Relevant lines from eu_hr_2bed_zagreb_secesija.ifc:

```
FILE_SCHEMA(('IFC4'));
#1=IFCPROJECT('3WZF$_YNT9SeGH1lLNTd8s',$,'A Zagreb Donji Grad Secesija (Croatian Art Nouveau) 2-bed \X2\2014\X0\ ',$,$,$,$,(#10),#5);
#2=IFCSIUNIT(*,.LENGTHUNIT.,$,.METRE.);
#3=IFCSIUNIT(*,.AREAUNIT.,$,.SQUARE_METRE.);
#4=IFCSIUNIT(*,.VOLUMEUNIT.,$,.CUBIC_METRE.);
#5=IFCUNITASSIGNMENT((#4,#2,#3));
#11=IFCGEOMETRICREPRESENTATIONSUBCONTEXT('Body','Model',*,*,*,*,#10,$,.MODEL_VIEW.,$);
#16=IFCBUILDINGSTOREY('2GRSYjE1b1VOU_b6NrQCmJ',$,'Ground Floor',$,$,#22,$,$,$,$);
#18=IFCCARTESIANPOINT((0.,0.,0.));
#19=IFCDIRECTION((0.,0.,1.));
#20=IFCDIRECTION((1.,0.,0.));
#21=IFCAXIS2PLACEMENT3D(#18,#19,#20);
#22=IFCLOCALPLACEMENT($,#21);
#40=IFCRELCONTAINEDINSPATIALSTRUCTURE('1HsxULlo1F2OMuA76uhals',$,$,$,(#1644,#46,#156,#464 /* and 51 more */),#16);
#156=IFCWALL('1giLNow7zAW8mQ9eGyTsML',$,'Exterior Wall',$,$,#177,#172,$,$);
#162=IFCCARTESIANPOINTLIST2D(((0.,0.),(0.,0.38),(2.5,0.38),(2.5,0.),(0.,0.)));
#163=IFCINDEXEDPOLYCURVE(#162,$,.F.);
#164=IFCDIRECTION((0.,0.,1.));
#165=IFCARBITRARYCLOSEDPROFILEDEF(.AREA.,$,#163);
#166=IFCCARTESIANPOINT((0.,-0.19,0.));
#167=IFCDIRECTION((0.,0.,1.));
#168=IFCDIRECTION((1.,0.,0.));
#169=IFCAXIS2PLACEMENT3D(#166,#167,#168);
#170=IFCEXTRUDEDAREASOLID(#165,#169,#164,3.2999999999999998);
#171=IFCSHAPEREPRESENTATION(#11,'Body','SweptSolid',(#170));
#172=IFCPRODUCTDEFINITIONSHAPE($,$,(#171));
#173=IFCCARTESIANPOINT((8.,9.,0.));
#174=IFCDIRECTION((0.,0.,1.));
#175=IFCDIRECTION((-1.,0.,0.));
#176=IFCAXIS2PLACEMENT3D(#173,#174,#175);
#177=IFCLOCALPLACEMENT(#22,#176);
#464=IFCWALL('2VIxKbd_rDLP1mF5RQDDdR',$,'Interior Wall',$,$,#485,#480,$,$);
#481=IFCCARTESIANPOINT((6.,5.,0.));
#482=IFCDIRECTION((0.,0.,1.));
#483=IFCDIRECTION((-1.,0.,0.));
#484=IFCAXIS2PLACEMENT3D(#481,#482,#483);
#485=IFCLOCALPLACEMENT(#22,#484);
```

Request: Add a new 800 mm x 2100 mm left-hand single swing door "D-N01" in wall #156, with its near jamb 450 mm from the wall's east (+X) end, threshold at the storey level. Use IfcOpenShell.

```python
import numpy as np
import ifcopenshell
import ifcopenshell.api.feature
import ifcopenshell.api.geometry
import ifcopenshell.api.root
import ifcopenshell.api.spatial
import ifcopenshell.geom
import ifcopenshell.util.element
import ifcopenshell.util.placement
import ifcopenshell.util.representation
import ifcopenshell.util.shape
import ifcopenshell.util.unit

model = ifcopenshell.open("eu_hr_2bed_zagreb_secesija.ifc")
unit_scale = ifcopenshell.util.unit.calculate_unit_scale(model)
settings = ifcopenshell.geom.settings()


def volume(element):
    """Net volume in cubic metres, openings subtracted."""
    shape = ifcopenshell.geom.create_shape(settings, element)
    return ifcopenshell.util.shape.get_volume(shape.geometry)


wall = model.by_guid("1giLNow7zAW8mQ9eGyTsML")
storey = ifcopenshell.util.element.get_container(wall, ifc_class="IfcBuildingStorey")
context = ifcopenshell.util.representation.get_context(model, "Model", "Body", "MODEL_VIEW")
before = volume(wall)

width, height, from_end, sill = 0.8, 2.1, 0.45, 0.0  # metres

# The wall runs along its own X axis, and the end named is its -X end.
wall_shape = ifcopenshell.geom.create_shape(settings, wall)
x, y, z = ifcopenshell.util.shape.get_vertices(wall_shape.geometry).T
start = x.min() + from_end
face, thickness = float(y.min()), float(y.max() - y.min())
wall_matrix = ifcopenshell.util.placement.get_local_placement(wall.ObjectPlacement)
level = ifcopenshell.util.placement.get_local_placement(storey.ObjectPlacement)[2, 3]


def in_wall(x, y):
    """Placement at x, y metres in the wall's axes, at sill height."""
    matrix = wall_matrix.copy()
    matrix[:, 3] = wall_matrix @ np.array([x / unit_scale, y / unit_scale, 0.0, 1.0])
    matrix[2, 3] = level + sill / unit_scale
    return matrix


# Opening: a box that overshoots both wall faces by 50 mm.
opening = ifcopenshell.api.root.create_entity(model, ifc_class="IfcOpeningElement", predefined_type="OPENING")
box = ifcopenshell.api.geometry.add_wall_representation(
    model, context=context, length=width, height=height, thickness=thickness + 0.1
)
ifcopenshell.api.geometry.assign_representation(model, product=opening, representation=box)
ifcopenshell.api.geometry.edit_object_placement(model, product=opening, matrix=in_wall(start, face - 0.05), is_si=False)
ifcopenshell.api.feature.add_feature(model, feature=opening, element=wall)

door = ifcopenshell.api.root.create_entity(model, ifc_class="IfcDoor", name="D-N01", predefined_type="DOOR")
door.OverallWidth, door.OverallHeight = width / unit_scale, height / unit_scale
door.OperationType = "SINGLE_SWING_LEFT"
body = ifcopenshell.api.geometry.add_door_representation(
    model,
    context=context,
    overall_width=door.OverallWidth,
    overall_height=door.OverallHeight,
    operation_type="SINGLE_SWING_LEFT",
    lining_properties={"LiningDepth": thickness / unit_scale, "ThresholdDepth": thickness / unit_scale},
)
ifcopenshell.api.geometry.assign_representation(model, product=door, representation=body)
ifcopenshell.api.spatial.assign_container(model, products=[door], relating_structure=storey)
ifcopenshell.api.feature.add_filling(model, opening=opening, element=door)

# The lining spans the wall, so the door starts at the wall face.
ifcopenshell.api.geometry.edit_object_placement(model, product=door, matrix=in_wall(start, face), is_si=False)

after = volume(wall)

print(f"wall volume {before:.3f} -> {after:.3f} m3")

model.write("eu_hr_2bed_zagreb_secesija-out.ifc")
```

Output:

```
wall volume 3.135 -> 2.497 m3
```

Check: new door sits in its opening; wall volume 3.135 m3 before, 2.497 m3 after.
